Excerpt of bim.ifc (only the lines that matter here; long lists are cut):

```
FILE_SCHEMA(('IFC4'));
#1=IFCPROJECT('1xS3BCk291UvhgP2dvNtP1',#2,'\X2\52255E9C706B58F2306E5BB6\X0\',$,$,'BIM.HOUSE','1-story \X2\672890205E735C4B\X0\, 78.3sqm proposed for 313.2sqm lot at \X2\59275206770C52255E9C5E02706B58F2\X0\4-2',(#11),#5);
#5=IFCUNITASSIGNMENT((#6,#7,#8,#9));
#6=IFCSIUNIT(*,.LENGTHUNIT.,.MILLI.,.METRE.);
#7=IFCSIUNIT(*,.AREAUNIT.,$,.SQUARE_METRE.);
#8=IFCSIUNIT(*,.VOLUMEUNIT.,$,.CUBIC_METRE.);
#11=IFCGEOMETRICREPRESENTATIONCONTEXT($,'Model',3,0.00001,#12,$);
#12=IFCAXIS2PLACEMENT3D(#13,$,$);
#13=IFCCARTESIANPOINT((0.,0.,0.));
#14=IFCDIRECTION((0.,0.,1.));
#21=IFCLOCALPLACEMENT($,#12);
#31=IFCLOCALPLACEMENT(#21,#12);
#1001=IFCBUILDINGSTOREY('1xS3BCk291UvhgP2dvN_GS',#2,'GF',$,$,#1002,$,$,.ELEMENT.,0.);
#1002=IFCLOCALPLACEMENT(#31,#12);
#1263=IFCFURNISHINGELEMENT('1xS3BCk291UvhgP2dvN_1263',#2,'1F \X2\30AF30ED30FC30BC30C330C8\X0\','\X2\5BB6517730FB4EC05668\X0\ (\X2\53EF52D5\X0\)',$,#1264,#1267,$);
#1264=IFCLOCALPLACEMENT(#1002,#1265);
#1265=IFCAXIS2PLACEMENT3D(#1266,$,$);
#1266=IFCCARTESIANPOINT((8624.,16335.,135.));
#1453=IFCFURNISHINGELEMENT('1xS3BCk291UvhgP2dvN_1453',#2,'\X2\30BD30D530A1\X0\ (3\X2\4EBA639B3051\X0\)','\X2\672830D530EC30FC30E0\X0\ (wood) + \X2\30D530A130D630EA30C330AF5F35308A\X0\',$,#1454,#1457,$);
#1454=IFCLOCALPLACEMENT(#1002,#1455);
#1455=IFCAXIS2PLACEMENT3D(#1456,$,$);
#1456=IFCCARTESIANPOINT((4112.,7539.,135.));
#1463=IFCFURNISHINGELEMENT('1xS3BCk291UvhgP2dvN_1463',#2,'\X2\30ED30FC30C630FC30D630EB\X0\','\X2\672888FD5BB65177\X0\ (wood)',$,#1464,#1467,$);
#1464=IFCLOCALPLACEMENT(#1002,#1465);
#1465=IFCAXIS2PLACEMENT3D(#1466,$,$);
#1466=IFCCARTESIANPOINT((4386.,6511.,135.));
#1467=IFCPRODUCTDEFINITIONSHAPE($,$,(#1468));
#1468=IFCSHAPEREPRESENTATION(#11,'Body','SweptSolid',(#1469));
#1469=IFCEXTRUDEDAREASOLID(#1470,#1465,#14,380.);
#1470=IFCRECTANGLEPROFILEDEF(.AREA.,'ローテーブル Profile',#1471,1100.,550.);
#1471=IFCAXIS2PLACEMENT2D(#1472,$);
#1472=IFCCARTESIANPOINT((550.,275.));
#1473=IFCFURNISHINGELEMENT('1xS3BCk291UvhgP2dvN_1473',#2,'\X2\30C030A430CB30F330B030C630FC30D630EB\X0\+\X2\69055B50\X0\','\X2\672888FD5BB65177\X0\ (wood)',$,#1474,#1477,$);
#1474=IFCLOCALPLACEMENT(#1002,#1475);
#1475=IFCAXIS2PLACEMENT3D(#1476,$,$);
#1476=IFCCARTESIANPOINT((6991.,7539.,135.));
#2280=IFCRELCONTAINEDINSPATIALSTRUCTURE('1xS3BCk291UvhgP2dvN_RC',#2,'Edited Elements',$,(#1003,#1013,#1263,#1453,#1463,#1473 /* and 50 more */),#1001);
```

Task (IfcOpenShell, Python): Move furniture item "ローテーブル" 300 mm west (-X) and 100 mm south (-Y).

```python
import ifcopenshell
import ifcopenshell.api.geometry
import ifcopenshell.util.placement
import ifcopenshell.util.unit

model = ifcopenshell.open("bim.ifc")
unit_scale = ifcopenshell.util.unit.calculate_unit_scale(model)

item = model.by_guid("1xS3BCk291UvhgP2dvN_1463")
matrix = ifcopenshell.util.placement.get_local_placement(item.ObjectPlacement)
matrix[0, 3] -= 0.3 / unit_scale
matrix[1, 3] -= 0.1 / unit_scale
ifcopenshell.api.geometry.edit_object_placement(model, product=item, matrix=matrix, is_si=False)

print(ifcopenshell.util.placement.get_local_placement(item.ObjectPlacement).round(3) + 0.0)

model.write("bim_updated.ifc")
```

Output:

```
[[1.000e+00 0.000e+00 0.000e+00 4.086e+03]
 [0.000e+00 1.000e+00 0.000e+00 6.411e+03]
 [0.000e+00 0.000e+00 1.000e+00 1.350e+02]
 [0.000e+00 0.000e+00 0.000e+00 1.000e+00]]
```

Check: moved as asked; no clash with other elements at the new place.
